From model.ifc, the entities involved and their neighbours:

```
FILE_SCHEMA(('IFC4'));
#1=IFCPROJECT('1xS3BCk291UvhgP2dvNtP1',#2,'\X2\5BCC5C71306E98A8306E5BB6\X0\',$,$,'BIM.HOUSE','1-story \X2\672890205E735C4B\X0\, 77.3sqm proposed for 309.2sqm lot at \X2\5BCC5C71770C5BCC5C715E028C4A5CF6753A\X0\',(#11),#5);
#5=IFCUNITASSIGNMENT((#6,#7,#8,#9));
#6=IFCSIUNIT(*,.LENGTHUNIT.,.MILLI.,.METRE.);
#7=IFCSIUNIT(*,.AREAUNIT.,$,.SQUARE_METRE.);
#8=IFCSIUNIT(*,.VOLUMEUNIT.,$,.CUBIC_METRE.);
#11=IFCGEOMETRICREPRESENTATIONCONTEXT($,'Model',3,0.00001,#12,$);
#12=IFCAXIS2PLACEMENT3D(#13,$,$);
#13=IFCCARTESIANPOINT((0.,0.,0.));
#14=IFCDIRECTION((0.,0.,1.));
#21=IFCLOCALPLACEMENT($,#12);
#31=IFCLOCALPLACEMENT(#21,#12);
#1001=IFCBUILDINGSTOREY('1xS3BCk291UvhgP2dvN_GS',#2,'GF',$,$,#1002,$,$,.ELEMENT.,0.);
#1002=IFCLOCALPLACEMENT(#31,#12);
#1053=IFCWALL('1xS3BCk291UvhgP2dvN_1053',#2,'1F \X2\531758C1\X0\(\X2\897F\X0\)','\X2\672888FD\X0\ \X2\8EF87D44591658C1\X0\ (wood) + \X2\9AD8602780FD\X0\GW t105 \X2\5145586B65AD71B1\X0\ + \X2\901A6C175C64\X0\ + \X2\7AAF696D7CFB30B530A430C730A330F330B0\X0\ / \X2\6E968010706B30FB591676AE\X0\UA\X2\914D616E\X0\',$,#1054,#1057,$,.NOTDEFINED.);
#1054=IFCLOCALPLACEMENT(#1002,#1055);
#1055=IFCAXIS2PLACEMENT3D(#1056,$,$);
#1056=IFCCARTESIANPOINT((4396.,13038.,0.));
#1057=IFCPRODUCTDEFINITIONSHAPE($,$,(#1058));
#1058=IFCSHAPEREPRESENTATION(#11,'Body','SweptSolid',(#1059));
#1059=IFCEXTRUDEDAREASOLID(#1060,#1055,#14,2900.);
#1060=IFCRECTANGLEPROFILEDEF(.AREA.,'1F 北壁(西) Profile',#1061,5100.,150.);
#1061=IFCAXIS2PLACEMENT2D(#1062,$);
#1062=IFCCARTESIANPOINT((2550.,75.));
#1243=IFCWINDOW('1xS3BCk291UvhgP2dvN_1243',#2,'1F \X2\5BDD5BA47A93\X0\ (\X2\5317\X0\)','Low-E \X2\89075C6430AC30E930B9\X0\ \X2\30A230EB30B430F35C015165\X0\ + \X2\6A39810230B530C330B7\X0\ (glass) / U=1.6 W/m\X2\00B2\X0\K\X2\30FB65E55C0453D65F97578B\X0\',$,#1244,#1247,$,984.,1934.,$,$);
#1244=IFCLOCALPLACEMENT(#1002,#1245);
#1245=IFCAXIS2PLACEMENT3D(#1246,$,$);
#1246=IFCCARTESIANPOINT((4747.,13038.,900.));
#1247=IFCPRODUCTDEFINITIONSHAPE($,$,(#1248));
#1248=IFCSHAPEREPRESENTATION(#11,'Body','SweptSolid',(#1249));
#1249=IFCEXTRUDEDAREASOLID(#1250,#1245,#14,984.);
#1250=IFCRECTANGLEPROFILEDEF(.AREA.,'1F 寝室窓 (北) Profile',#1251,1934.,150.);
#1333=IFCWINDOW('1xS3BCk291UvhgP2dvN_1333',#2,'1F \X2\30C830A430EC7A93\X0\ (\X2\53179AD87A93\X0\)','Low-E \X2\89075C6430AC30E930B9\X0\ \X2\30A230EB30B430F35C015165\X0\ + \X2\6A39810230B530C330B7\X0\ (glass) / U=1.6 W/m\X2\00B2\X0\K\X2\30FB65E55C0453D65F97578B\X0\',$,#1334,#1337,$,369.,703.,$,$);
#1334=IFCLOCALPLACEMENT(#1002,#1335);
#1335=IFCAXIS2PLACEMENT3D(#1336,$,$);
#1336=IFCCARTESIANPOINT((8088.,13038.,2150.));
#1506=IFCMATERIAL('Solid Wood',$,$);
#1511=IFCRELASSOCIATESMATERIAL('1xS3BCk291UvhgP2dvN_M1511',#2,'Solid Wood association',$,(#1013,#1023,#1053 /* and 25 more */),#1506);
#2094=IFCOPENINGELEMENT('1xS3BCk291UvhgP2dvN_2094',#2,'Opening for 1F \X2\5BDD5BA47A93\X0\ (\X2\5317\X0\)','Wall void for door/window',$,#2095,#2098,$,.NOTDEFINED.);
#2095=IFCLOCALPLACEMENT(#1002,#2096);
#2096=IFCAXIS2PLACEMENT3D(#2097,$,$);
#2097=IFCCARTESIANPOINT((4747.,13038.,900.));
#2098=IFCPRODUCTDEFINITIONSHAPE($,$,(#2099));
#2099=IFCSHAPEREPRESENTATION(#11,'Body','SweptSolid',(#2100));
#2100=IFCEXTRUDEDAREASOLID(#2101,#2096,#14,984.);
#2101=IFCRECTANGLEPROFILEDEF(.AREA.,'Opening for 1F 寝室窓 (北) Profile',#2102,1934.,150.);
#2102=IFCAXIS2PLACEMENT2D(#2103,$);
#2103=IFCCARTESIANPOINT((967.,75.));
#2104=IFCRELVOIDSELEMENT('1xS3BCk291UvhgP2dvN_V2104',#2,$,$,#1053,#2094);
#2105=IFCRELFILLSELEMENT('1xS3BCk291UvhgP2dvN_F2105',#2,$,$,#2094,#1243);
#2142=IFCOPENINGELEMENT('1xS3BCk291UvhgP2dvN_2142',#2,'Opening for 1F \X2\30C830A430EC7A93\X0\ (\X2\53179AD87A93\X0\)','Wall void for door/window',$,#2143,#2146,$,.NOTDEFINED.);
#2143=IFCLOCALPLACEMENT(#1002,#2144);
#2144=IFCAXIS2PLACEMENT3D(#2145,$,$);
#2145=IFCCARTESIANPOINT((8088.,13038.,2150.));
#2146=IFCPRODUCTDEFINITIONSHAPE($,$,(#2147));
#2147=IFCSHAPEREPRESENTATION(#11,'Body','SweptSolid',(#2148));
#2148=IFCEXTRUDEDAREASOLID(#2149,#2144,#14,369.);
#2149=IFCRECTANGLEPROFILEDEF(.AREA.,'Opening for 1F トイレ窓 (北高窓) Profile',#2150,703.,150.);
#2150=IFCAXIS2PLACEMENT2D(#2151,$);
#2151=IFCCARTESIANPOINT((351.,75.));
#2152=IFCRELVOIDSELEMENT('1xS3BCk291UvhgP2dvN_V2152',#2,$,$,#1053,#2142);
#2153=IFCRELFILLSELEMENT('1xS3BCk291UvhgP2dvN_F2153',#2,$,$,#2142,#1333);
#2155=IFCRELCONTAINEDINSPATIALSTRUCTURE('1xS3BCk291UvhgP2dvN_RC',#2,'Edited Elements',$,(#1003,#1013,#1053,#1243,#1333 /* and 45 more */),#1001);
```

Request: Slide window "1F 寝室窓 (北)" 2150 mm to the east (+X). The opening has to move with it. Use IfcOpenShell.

```python
import ifcopenshell
import ifcopenshell.api.geometry
import ifcopenshell.util.placement

model = ifcopenshell.open("model.ifc")

window = model.by_id(1243)
opening = window.FillsVoids[0].RelatingOpeningElement
wall = opening.VoidsElements[0].RelatingBuildingElement

wall_matrix = ifcopenshell.util.placement.get_local_placement(wall.ObjectPlacement)
shift = wall_matrix[:3, 0] * 2150.0
before = ifcopenshell.util.placement.get_local_placement(window.ObjectPlacement)[:3, 3].copy()

# The window is not placed relative to its opening, so move both.
for product in (opening, window):
    matrix = ifcopenshell.util.placement.get_local_placement(product.ObjectPlacement)
    matrix[:3, 3] += shift
    ifcopenshell.api.geometry.edit_object_placement(model, product=product, matrix=matrix, is_si=False)

after = ifcopenshell.util.placement.get_local_placement(window.ObjectPlacement)[:3, 3]
print("window moved by", (after - before).round(3) + 0.0)

model.write("model_rev.ifc")
```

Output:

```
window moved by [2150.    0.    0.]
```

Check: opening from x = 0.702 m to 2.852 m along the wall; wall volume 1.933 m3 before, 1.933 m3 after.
